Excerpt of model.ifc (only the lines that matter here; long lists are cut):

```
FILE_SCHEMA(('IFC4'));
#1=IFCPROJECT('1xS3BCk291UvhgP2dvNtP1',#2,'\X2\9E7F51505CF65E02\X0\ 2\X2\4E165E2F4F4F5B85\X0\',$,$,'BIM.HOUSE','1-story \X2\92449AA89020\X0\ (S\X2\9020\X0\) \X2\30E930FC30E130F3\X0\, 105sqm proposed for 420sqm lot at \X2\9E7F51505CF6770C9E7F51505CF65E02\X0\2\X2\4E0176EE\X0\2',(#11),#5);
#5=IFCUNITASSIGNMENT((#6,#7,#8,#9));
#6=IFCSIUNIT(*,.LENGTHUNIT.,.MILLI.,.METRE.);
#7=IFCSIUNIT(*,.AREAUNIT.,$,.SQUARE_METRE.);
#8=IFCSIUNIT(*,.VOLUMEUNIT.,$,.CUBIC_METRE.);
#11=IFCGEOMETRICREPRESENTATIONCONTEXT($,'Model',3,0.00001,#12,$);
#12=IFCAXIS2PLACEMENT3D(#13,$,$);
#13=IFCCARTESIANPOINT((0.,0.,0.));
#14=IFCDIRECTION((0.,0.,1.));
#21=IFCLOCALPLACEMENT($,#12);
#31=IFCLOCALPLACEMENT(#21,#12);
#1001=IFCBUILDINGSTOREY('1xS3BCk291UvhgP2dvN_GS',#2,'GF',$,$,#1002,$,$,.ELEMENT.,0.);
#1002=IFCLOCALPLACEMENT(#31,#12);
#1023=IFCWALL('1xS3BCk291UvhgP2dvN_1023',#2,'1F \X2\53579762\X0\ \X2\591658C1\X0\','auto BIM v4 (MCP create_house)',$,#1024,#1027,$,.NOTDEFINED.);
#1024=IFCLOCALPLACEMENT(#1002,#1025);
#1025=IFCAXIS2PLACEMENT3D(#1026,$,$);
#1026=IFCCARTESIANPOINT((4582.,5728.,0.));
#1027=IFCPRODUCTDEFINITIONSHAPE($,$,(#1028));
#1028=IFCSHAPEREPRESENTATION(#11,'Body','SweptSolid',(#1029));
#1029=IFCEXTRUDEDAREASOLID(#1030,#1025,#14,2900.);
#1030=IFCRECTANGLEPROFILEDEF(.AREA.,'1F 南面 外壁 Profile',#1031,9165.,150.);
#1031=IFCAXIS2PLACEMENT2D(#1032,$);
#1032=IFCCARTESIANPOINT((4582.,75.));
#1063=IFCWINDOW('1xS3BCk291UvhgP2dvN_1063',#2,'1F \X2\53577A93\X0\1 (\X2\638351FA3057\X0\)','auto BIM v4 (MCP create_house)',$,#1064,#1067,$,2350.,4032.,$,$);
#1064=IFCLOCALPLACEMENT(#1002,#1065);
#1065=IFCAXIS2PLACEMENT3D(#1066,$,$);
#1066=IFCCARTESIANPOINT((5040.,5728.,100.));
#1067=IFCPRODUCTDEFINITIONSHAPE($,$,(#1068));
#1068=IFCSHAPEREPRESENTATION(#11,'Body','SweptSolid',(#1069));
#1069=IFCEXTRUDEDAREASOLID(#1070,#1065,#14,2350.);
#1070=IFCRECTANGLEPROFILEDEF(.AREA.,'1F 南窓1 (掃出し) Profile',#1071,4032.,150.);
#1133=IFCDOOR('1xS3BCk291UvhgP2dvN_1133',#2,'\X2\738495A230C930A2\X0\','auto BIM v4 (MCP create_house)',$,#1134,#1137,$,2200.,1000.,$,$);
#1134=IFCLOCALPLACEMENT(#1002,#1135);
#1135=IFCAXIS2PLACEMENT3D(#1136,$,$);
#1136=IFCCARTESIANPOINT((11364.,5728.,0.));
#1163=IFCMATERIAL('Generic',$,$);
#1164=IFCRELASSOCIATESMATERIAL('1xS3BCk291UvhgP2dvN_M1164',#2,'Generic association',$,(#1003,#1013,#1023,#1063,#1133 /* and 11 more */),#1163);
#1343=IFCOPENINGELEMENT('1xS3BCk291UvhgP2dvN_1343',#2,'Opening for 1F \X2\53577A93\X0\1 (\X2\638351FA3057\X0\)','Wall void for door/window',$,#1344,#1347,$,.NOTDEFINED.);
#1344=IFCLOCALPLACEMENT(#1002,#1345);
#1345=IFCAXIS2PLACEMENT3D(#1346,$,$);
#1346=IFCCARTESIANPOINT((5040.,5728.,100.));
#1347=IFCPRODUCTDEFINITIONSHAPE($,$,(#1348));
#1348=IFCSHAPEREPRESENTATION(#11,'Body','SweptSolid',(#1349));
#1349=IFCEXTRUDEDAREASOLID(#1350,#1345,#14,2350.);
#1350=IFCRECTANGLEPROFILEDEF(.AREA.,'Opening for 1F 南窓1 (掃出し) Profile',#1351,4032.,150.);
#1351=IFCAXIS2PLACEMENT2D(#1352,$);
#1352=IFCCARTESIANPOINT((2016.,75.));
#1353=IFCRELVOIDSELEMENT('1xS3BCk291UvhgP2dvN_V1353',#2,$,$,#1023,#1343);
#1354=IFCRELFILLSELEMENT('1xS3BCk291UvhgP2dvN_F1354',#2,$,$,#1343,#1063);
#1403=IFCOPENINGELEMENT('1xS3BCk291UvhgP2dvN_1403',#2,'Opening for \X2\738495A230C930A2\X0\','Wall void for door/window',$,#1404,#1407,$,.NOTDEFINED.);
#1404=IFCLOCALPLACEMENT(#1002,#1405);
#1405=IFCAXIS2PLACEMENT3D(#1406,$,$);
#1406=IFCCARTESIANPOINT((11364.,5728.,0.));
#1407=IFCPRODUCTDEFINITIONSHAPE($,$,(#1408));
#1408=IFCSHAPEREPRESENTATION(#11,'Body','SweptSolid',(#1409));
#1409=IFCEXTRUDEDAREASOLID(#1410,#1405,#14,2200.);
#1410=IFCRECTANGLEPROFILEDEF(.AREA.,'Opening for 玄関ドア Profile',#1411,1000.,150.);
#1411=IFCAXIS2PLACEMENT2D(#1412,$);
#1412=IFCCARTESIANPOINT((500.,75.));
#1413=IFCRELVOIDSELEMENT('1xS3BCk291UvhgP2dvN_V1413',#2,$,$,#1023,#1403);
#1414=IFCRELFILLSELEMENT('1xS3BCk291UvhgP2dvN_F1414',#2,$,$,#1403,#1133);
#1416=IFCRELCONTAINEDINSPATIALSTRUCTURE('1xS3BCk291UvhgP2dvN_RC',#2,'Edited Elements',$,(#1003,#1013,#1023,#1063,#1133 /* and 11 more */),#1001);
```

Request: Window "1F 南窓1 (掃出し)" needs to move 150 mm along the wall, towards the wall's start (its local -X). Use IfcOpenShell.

```python
import ifcopenshell
import ifcopenshell.api.geometry
import ifcopenshell.util.placement
import ifcopenshell.util.unit

model = ifcopenshell.open("model.ifc")
unit_scale = ifcopenshell.util.unit.calculate_unit_scale(model)

window = model.by_id(1063)
opening = window.FillsVoids[0].RelatingOpeningElement
wall = opening.VoidsElements[0].RelatingBuildingElement

wall_matrix = ifcopenshell.util.placement.get_local_placement(wall.ObjectPlacement)
shift = wall_matrix[:3, 0] * -0.15 / unit_scale
before = ifcopenshell.util.placement.get_local_placement(window.ObjectPlacement)[:3, 3].copy()

# The window is not placed relative to its opening, so move both.
for product in (opening, window):
    matrix = ifcopenshell.util.placement.get_local_placement(product.ObjectPlacement)
    matrix[:3, 3] += shift
    ifcopenshell.api.geometry.edit_object_placement(model, product=product, matrix=matrix, is_si=False)

after = ifcopenshell.util.placement.get_local_placement(window.ObjectPlacement)[:3, 3]
print("window moved by", (after - before).round(3) + 0.0)

model.write("model_rev.ifc")
```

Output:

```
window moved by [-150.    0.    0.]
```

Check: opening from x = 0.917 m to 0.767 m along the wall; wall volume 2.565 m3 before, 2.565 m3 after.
